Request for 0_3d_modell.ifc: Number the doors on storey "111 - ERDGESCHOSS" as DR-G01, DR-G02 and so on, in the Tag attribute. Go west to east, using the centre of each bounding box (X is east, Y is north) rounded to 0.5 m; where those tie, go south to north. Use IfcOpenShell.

First a look at what the model holds.

```python
import ifcopenshell
import ifcopenshell.util.element
import ifcopenshell.util.placement

model = ifcopenshell.open("0_3d_modell.ifc")
print(model.schema)
storey = next(s for s in model.by_type("IfcBuildingStorey") if s.Name == "111 - ERDGESCHOSS")
doors = [e for e in ifcopenshell.util.element.get_decomposition(storey) if e.is_a("IfcDoor")]
for e in sorted(doors, key=lambda e: e.id()):
    origin = ifcopenshell.util.placement.get_local_placement(e.ObjectPlacement)[:3, 3]
    print(e.id(), e.Tag, e.Name, origin.round(2) + 0.0, sep=" | ")
```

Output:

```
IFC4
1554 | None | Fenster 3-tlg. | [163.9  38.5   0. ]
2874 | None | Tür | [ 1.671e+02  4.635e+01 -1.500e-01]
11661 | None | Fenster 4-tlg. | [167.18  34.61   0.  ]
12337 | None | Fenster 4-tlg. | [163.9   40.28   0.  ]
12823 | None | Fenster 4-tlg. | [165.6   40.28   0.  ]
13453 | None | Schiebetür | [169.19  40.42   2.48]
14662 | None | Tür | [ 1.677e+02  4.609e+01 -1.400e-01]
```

```python
import ifcopenshell
import ifcopenshell.geom
import ifcopenshell.util.element
import ifcopenshell.util.shape

model = ifcopenshell.open("0_3d_modell.ifc")
settings = ifcopenshell.geom.settings()
settings.set("use-world-coords", True)


def centre(element):
    shape = ifcopenshell.geom.create_shape(settings, element)
    return ifcopenshell.util.shape.get_bbox_centroid(shape.geometry)


storey = next(s for s in model.by_type("IfcBuildingStorey") if s.Name == "111 - ERDGESCHOSS")
doors = [e for e in ifcopenshell.util.element.get_decomposition(storey) if e.is_a("IfcDoor")]

# Insertion points can sit at a corner or the storey origin, so sort by the geometry (in metres).
centres = {e: centre(e) for e in doors}
doors.sort(key=lambda e: (round(centres[e][0] / 0.5), centres[e][1]))

for i, e in enumerate(doors, start=1):
    number = f"DR-G{i:02d}"
    e.Tag = number
    print(e.id(), number)

model.write("0_3d_modell_rev.ifc")
```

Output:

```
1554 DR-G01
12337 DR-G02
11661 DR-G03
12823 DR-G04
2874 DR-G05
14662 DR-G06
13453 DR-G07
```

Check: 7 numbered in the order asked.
